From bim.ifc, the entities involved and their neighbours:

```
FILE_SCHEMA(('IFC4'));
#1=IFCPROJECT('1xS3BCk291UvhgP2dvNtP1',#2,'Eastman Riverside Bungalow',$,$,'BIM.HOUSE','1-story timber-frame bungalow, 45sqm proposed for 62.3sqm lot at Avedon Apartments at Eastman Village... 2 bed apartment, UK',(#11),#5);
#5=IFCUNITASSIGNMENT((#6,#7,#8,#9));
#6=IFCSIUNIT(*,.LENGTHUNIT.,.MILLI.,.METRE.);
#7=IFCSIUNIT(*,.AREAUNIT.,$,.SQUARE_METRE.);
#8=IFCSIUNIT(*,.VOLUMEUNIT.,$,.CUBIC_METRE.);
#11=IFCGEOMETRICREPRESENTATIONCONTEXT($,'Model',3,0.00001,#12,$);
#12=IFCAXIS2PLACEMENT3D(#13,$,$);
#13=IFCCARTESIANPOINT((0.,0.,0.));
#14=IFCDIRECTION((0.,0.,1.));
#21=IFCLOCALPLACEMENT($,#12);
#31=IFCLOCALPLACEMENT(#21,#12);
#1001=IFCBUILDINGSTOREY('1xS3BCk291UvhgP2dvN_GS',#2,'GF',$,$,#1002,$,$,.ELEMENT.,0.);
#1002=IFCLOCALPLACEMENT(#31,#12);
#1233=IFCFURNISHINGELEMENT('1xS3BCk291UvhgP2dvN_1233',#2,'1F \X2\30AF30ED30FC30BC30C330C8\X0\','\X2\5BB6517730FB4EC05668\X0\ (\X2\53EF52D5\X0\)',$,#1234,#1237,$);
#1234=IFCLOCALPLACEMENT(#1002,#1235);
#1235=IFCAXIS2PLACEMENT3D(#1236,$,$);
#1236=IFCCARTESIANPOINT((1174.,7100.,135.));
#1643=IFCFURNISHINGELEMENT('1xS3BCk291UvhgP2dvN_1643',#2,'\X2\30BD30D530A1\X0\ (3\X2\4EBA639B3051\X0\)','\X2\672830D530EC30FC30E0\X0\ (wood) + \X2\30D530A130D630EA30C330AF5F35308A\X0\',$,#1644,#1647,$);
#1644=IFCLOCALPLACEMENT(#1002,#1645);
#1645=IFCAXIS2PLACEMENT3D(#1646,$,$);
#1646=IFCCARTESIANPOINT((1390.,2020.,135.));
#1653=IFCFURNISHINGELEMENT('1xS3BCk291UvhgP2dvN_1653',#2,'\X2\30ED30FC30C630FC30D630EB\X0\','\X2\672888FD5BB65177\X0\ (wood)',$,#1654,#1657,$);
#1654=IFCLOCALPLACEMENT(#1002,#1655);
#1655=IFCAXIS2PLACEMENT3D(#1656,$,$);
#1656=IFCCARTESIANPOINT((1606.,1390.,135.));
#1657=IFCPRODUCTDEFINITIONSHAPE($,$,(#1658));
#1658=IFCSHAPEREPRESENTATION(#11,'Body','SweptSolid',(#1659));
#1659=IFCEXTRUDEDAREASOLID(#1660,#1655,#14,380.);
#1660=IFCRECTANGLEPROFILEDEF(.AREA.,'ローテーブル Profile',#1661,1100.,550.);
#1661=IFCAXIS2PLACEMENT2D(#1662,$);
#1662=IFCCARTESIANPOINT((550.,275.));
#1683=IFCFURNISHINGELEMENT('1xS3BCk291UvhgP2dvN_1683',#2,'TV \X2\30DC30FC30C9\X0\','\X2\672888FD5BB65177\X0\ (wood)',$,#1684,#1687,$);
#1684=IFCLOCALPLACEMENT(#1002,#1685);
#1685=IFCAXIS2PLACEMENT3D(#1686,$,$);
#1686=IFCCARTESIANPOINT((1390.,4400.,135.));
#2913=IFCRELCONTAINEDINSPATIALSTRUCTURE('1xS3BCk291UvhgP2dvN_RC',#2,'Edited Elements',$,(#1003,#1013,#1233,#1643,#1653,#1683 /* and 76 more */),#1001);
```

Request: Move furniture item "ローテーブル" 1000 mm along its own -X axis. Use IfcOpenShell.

```python
import ifcopenshell
import ifcopenshell.api.geometry
import ifcopenshell.util.placement
import ifcopenshell.util.unit

model = ifcopenshell.open("bim.ifc")
unit_scale = ifcopenshell.util.unit.calculate_unit_scale(model)

item = model.by_guid("1xS3BCk291UvhgP2dvN_1653")
matrix = ifcopenshell.util.placement.get_local_placement(item.ObjectPlacement)
matrix[:3, 3] -= matrix[:3, 0] * 1 / unit_scale
ifcopenshell.api.geometry.edit_object_placement(model, product=item, matrix=matrix, is_si=False)

print(ifcopenshell.util.placement.get_local_placement(item.ObjectPlacement).round(3) + 0.0)

model.write("bim-out.ifc")
```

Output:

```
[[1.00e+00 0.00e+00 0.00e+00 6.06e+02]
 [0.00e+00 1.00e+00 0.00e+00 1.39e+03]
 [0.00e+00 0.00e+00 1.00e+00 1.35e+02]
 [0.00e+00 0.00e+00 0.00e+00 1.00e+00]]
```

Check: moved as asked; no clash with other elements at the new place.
